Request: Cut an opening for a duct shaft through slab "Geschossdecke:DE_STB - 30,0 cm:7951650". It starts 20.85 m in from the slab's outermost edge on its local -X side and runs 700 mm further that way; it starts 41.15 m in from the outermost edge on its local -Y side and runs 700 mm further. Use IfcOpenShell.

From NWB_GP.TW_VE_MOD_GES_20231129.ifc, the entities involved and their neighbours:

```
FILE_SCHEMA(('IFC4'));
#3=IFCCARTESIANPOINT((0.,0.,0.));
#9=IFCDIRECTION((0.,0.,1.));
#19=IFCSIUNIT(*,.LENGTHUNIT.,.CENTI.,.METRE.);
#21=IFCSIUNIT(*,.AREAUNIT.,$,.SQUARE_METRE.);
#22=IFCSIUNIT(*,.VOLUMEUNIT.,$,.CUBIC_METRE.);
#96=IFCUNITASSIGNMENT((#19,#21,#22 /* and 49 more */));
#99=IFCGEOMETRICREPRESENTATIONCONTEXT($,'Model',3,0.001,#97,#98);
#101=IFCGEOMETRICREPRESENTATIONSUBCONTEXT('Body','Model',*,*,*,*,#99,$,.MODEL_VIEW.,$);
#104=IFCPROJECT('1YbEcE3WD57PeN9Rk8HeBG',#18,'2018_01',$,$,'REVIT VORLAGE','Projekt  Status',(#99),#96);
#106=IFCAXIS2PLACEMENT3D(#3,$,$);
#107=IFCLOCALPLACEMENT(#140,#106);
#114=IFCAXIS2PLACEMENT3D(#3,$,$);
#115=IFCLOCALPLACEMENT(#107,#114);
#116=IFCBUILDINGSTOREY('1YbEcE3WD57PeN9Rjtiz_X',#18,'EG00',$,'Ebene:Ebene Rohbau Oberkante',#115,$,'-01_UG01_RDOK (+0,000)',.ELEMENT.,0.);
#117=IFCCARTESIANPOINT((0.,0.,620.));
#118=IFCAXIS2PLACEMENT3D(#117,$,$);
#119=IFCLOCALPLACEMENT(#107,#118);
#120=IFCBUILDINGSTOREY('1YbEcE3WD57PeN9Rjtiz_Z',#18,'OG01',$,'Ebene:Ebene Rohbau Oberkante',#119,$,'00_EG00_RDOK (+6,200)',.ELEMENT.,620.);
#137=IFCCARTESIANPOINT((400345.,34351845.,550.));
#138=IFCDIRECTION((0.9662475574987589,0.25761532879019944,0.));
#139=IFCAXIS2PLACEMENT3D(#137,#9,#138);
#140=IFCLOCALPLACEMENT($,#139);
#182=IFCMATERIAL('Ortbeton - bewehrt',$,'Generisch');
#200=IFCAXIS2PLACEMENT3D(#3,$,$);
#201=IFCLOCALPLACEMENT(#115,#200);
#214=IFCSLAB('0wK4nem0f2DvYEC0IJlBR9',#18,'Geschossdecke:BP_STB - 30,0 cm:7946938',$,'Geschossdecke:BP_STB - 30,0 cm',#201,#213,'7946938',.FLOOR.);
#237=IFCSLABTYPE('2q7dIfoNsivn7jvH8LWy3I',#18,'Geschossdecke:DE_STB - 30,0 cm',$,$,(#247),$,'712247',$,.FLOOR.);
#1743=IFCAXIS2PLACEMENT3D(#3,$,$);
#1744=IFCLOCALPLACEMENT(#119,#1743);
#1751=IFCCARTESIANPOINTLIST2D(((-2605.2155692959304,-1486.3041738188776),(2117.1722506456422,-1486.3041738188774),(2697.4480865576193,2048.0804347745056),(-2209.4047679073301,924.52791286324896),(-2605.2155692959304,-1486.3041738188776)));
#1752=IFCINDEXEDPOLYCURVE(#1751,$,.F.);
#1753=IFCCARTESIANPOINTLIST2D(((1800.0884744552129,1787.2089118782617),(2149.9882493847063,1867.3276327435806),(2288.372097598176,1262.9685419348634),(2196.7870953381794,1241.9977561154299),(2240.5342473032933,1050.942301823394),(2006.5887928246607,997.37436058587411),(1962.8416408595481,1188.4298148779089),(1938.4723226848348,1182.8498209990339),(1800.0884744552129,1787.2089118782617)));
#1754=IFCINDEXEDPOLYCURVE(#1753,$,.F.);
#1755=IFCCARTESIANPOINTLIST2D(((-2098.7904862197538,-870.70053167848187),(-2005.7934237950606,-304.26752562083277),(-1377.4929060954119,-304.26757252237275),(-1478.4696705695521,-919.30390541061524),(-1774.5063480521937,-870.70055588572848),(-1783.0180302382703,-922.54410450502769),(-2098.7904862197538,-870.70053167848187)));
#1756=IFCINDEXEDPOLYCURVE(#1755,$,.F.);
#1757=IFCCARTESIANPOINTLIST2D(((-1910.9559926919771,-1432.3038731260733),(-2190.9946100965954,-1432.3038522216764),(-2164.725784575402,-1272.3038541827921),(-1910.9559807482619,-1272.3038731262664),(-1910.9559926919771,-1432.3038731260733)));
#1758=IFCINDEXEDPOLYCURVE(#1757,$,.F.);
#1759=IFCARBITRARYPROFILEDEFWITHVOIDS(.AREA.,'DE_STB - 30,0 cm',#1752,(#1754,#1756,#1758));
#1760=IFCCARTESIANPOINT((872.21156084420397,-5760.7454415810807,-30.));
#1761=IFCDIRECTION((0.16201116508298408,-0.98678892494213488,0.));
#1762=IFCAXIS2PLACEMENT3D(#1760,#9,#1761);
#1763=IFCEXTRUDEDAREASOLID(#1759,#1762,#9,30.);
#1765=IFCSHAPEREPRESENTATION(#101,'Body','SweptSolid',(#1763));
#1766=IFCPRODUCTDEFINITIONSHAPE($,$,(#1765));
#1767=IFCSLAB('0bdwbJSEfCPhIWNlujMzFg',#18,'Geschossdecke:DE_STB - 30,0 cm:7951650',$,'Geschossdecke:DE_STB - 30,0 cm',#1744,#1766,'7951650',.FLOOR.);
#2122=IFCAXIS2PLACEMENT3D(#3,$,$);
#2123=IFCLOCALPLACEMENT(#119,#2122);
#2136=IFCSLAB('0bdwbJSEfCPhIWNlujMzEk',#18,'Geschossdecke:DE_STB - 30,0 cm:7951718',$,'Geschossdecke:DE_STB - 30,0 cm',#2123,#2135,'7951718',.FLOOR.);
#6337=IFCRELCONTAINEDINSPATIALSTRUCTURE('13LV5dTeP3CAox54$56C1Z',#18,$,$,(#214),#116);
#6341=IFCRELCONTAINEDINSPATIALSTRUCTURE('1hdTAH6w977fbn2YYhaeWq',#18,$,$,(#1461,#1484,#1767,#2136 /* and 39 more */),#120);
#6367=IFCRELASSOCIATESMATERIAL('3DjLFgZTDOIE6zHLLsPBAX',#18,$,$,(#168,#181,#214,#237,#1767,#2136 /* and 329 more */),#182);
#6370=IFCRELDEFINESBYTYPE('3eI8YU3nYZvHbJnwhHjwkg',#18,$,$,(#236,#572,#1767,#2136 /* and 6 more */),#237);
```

```python
import numpy as np
import ifcopenshell
import ifcopenshell.api.feature
import ifcopenshell.api.geometry
import ifcopenshell.api.root
import ifcopenshell.geom
import ifcopenshell.util.placement
import ifcopenshell.util.representation
import ifcopenshell.util.shape
import ifcopenshell.util.unit

model = ifcopenshell.open("NWB_GP.TW_VE_MOD_GES_20231129.ifc")
unit_scale = ifcopenshell.util.unit.calculate_unit_scale(model)
settings = ifcopenshell.geom.settings()


def volume(element):
    """Net volume in cubic metres, openings subtracted."""
    shape = ifcopenshell.geom.create_shape(settings, element)
    return ifcopenshell.util.shape.get_volume(shape.geometry)


slab = model.by_guid("0bdwbJSEfCPhIWNlujMzFg")
before = volume(slab)

# Extent in the slab's own axes, in metres. The edges named are its -X and -Y sides.
slab_shape = ifcopenshell.geom.create_shape(settings, slab)
vertices = ifcopenshell.util.shape.get_vertices(slab_shape.geometry)
x_min, y_min, bottom = vertices.min(axis=0)
top = vertices[:, 2].max()

opening = ifcopenshell.api.root.create_entity(model, ifc_class="IfcOpeningElement", name="Duct shaft opening", predefined_type="OPENING")
context = ifcopenshell.util.representation.get_context(model, "Model", "Body", "MODEL_VIEW")
width, depth = 0.7, 0.7
outline = [(0.0, 0.0), (width, 0.0), (width, depth), (0.0, depth), (0.0, 0.0)]
# Overshoot both faces by 50 mm so the cut is clean.
shape = ifcopenshell.api.geometry.add_slab_representation(
    model, context=context, depth=top - bottom + 0.1, polyline=outline
)
ifcopenshell.api.geometry.assign_representation(model, product=opening, representation=shape)

matrix = ifcopenshell.util.placement.get_local_placement(slab.ObjectPlacement)
matrix[:, 3] = matrix @ np.append(np.array([x_min + 20.85, y_min + 41.15, bottom - 0.05]) / unit_scale, 1.0)
ifcopenshell.api.geometry.edit_object_placement(model, product=opening, matrix=matrix, is_si=False)
ifcopenshell.api.feature.add_feature(model, feature=opening, element=slab)

after = volume(slab)

print(f"slab volume {before:.3f} -> {after:.3f} m3")

model.write("NWB_GP.TW_VE_MOD_GES_20231129_updated.ifc")
```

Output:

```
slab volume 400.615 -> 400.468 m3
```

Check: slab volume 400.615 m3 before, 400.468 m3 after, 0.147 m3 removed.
